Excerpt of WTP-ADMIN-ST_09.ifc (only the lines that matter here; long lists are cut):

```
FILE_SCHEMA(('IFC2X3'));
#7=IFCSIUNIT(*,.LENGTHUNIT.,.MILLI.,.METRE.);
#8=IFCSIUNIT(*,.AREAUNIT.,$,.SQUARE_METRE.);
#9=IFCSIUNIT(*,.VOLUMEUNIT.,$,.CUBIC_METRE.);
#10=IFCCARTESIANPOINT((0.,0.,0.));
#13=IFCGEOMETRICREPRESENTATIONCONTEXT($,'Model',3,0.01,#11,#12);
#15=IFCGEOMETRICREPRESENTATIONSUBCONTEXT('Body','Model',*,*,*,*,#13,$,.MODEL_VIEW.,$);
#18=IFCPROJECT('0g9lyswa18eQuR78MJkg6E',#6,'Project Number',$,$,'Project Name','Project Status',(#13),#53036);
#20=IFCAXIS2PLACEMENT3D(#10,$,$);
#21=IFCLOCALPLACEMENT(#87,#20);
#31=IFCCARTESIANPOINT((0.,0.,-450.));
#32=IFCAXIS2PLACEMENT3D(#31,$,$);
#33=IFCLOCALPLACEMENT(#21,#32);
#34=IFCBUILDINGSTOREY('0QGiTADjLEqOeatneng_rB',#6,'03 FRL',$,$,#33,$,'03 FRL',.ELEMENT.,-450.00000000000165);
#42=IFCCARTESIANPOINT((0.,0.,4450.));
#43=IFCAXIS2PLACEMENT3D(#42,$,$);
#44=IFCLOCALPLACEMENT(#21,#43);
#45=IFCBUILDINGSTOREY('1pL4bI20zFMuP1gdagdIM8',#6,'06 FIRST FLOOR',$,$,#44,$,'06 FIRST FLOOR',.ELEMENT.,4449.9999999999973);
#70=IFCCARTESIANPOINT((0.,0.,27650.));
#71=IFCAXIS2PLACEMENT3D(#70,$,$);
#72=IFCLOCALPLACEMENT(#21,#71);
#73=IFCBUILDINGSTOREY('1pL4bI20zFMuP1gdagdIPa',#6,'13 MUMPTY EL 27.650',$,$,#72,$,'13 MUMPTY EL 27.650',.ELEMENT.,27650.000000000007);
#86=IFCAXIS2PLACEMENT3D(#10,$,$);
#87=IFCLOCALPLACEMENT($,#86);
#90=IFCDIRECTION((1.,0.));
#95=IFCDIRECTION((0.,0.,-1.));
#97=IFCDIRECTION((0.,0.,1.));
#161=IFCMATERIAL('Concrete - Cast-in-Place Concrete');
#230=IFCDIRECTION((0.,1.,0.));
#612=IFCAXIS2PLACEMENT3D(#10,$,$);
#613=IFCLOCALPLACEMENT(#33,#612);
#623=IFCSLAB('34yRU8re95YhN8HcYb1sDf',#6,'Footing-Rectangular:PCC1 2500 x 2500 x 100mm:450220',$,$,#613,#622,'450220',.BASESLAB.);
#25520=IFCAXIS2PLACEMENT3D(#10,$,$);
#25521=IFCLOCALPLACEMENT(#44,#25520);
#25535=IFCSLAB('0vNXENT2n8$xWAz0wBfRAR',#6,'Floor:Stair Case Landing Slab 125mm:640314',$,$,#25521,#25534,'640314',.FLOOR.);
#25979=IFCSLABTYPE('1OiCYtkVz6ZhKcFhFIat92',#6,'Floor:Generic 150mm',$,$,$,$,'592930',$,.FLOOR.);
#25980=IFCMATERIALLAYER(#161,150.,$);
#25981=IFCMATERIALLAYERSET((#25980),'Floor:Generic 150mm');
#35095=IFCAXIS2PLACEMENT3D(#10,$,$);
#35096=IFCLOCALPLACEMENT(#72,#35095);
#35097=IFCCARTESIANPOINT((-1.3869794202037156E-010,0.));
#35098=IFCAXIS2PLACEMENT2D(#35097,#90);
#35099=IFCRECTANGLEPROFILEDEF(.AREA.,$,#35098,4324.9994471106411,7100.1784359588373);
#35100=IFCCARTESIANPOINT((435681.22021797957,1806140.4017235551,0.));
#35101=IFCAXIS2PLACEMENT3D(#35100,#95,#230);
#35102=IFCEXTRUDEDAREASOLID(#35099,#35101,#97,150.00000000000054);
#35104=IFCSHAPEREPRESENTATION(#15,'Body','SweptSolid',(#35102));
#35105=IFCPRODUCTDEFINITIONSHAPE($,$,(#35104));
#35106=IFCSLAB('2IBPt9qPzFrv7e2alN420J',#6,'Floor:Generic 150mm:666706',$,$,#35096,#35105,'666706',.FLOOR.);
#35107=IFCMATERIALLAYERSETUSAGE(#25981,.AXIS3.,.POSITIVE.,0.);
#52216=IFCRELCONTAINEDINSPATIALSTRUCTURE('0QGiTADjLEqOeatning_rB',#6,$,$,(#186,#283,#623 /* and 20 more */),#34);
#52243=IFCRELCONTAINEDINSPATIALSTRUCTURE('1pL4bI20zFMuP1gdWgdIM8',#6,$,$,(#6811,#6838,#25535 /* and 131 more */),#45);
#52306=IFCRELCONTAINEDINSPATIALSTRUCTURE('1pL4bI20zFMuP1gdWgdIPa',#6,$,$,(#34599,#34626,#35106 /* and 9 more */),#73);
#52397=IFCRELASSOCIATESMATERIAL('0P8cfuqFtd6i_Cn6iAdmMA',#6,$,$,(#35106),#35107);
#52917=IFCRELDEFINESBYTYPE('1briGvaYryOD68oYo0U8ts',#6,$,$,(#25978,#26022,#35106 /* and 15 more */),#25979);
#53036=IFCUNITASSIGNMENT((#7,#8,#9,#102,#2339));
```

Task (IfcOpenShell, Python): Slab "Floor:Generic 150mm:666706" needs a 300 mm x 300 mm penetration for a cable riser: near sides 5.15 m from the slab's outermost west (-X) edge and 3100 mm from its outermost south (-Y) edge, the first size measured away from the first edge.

```python
import numpy as np
import ifcopenshell
import ifcopenshell.api.feature
import ifcopenshell.api.geometry
import ifcopenshell.api.root
import ifcopenshell.geom
import ifcopenshell.util.placement
import ifcopenshell.util.representation
import ifcopenshell.util.shape
import ifcopenshell.util.unit

model = ifcopenshell.open("WTP-ADMIN-ST_09.ifc")
unit_scale = ifcopenshell.util.unit.calculate_unit_scale(model)
settings = ifcopenshell.geom.settings()


def volume(element):
    """Net volume in cubic metres, openings subtracted."""
    shape = ifcopenshell.geom.create_shape(settings, element)
    return ifcopenshell.util.shape.get_volume(shape.geometry)


slab = model.by_guid("2IBPt9qPzFrv7e2alN420J")
before = volume(slab)

# Extent in the slab's own axes, in metres. The edges named are its -X and -Y sides.
slab_shape = ifcopenshell.geom.create_shape(settings, slab)
vertices = ifcopenshell.util.shape.get_vertices(slab_shape.geometry)
x_min, y_min, bottom = vertices.min(axis=0)
top = vertices[:, 2].max()

opening = ifcopenshell.api.root.create_entity(model, ifc_class="IfcOpeningElement", name="Cable riser opening")
context = ifcopenshell.util.representation.get_context(model, "Model", "Body", "MODEL_VIEW")
width, depth = 0.3, 0.3
outline = [(0.0, 0.0), (width, 0.0), (width, depth), (0.0, depth), (0.0, 0.0)]
# Overshoot both faces by 50 mm so the cut is clean.
shape = ifcopenshell.api.geometry.add_slab_representation(
    model, context=context, depth=top - bottom + 0.1, polyline=outline
)
ifcopenshell.api.geometry.assign_representation(model, product=opening, representation=shape)

matrix = ifcopenshell.util.placement.get_local_placement(slab.ObjectPlacement)
matrix[:, 3] = matrix @ np.append(np.array([x_min + 5.15, y_min + 3.1, bottom - 0.05]) / unit_scale, 1.0)
ifcopenshell.api.geometry.edit_object_placement(model, product=opening, matrix=matrix, is_si=False)
ifcopenshell.api.feature.add_feature(model, feature=opening, element=slab)

after = volume(slab)

print(f"slab volume {before:.3f} -> {after:.3f} m3")

model.write("WTP-ADMIN-ST_09-out.ifc")
```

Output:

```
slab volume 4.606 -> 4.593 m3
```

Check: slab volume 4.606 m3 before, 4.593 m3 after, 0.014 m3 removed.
